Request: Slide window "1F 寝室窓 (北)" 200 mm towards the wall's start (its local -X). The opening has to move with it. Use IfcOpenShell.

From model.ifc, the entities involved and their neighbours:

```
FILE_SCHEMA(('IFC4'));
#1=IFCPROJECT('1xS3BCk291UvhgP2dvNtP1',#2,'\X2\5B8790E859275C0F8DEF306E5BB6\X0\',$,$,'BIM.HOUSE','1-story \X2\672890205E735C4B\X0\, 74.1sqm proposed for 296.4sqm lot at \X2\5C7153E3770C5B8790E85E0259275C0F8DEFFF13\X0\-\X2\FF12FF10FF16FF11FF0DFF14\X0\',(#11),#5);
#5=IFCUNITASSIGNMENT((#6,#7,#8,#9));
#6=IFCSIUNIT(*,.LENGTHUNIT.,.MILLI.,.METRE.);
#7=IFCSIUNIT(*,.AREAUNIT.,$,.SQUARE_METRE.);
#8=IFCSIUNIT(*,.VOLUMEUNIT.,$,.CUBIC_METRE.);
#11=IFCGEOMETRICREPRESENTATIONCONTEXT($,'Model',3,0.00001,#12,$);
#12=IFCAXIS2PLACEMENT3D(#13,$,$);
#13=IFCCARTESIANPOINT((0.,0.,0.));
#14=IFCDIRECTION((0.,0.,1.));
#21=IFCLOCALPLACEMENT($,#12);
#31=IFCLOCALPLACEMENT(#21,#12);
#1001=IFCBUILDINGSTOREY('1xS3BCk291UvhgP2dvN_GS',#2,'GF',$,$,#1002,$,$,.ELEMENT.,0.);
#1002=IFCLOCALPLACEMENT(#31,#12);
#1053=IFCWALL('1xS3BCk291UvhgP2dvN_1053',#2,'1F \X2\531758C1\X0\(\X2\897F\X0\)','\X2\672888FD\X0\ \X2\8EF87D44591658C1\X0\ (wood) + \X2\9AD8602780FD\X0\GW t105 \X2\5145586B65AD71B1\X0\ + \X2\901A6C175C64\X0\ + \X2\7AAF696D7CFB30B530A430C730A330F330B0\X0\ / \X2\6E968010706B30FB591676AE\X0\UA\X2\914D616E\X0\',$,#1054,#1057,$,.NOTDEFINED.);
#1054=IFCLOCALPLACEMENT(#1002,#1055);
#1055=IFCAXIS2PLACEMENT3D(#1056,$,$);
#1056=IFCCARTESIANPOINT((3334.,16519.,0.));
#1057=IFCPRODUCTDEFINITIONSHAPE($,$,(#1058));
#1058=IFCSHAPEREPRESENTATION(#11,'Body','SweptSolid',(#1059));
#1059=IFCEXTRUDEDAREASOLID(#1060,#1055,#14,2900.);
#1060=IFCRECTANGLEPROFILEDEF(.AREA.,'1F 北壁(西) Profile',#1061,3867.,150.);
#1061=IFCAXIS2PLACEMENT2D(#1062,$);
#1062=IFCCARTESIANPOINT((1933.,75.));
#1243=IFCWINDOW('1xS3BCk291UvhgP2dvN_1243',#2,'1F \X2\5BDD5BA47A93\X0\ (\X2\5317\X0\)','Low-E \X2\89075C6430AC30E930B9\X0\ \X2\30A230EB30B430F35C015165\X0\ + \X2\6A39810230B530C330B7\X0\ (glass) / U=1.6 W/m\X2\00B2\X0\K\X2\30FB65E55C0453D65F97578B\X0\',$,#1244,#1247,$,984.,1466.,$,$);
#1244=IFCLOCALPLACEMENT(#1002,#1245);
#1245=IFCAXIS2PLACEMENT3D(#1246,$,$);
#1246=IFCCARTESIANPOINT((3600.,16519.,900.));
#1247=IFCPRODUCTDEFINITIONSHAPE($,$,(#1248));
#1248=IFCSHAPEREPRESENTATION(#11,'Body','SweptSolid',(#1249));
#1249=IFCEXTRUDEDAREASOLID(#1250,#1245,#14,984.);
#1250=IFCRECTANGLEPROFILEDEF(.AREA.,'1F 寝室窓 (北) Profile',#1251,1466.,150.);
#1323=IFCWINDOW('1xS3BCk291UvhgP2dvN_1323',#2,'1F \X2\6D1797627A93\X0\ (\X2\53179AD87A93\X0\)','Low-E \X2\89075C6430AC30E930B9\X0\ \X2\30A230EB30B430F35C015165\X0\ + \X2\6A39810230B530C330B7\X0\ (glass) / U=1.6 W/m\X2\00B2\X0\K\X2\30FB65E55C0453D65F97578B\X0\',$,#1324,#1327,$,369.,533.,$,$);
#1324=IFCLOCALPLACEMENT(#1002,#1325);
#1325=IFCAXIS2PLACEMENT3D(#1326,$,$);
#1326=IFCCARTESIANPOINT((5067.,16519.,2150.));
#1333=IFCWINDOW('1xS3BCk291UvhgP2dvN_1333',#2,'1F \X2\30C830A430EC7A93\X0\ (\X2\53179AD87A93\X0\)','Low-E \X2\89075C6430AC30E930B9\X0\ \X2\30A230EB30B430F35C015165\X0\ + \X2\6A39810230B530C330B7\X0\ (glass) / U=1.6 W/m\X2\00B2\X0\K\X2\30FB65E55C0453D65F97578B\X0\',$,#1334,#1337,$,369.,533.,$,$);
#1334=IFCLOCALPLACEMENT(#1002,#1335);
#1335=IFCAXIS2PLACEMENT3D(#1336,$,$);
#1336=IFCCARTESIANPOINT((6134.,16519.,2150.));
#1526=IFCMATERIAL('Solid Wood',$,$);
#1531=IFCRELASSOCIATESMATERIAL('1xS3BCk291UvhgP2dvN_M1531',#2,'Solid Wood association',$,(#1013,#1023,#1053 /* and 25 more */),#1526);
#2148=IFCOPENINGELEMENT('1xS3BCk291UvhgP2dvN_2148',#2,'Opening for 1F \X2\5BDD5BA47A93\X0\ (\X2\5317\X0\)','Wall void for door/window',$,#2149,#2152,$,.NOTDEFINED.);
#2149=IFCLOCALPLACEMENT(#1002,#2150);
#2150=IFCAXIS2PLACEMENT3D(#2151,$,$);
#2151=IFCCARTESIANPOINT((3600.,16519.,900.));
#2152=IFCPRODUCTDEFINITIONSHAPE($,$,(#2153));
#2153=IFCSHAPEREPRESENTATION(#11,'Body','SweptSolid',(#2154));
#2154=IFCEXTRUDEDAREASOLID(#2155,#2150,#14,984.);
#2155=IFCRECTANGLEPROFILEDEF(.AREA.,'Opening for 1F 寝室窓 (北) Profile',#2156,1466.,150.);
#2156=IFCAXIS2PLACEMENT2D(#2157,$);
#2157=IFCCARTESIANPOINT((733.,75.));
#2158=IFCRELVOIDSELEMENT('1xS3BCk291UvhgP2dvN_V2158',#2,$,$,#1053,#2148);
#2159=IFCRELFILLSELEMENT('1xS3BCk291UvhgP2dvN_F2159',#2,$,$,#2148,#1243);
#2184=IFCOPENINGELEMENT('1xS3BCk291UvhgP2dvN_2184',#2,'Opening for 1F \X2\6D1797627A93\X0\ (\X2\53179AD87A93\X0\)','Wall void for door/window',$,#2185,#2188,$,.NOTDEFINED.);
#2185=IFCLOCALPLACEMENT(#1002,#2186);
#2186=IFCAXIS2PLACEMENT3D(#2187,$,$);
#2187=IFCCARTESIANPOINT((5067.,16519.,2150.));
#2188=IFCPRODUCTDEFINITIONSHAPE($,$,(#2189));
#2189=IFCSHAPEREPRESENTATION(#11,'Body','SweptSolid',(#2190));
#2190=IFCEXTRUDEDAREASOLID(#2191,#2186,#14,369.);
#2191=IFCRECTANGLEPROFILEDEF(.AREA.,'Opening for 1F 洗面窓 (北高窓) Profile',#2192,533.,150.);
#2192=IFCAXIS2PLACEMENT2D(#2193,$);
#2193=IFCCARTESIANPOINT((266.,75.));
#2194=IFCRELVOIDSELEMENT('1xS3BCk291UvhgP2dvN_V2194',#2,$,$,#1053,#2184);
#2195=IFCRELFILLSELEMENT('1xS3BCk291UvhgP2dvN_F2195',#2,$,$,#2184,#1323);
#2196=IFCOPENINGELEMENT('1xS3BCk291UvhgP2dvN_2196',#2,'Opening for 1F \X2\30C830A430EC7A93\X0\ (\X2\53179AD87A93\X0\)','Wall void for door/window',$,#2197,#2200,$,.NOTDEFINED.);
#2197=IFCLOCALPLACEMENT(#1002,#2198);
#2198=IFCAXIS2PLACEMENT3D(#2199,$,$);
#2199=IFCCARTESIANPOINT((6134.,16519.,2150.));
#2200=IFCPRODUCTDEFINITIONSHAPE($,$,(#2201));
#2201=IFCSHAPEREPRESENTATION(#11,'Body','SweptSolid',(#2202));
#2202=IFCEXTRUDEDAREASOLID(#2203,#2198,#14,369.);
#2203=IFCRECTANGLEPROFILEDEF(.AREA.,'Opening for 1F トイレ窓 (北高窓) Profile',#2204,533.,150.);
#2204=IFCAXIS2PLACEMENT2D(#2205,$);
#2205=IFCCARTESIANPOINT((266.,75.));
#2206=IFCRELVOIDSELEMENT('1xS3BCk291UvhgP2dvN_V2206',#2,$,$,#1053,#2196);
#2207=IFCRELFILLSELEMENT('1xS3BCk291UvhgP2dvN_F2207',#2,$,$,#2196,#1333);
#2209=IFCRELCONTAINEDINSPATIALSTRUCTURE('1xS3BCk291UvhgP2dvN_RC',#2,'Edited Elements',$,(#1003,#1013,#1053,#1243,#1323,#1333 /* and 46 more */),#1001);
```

```python
import ifcopenshell
import ifcopenshell.api.geometry
import ifcopenshell.util.placement

model = ifcopenshell.open("model.ifc")

window = model.by_guid("1xS3BCk291UvhgP2dvN_1243")
opening = window.FillsVoids[0].RelatingOpeningElement
wall = opening.VoidsElements[0].RelatingBuildingElement

wall_matrix = ifcopenshell.util.placement.get_local_placement(wall.ObjectPlacement)
shift = wall_matrix[:3, 0] * -200.0
before = ifcopenshell.util.placement.get_local_placement(window.ObjectPlacement)[:3, 3].copy()

# The window is not placed relative to its opening, so move both.
for product in (opening, window):
    matrix = ifcopenshell.util.placement.get_local_placement(product.ObjectPlacement)
    matrix[:3, 3] += shift
    ifcopenshell.api.geometry.edit_object_placement(model, product=product, matrix=matrix, is_si=False)

after = ifcopenshell.util.placement.get_local_placement(window.ObjectPlacement)[:3, 3]
print("window moved by", (after - before).round(3) + 0.0)

model.write("model_v2.ifc")
```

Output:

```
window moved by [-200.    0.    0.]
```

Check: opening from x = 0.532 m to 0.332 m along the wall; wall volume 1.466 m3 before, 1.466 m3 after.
